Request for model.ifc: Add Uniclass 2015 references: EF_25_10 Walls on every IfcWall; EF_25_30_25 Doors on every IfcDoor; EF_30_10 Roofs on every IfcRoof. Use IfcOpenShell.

First a look at what the model holds.

```python
import ifcopenshell

model = ifcopenshell.open("model.ifc")
print(model.schema)
print("classifications:", [c.Name for c in model.by_type("IfcClassification")])
for ifc_class in ("IfcDoor", "IfcRoof", "IfcStair", "IfcWall", "IfcWindow"):
    print(ifc_class, len(model.by_type(ifc_class)))
```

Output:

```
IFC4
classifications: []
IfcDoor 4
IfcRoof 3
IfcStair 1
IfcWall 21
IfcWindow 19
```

```python
import ifcopenshell
import ifcopenshell.api.classification

model = ifcopenshell.open("model.ifc")

system = ifcopenshell.api.classification.add_classification(model, classification="Uniclass 2015")

codes = {
    "IfcWall": ("EF_25_10", "Walls"),
    "IfcDoor": ("EF_25_30_25", "Doors"),
    "IfcRoof": ("EF_30_10", "Roofs"),
}
for ifc_class, (code, name) in codes.items():
    products = model.by_type(ifc_class)
    ifcopenshell.api.classification.add_reference(
        model, products=products, classification=system, identification=code, name=name
    )
    print(code, len(products))

model.write("model_rev.ifc")
```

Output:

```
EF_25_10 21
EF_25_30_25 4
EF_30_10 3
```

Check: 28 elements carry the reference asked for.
